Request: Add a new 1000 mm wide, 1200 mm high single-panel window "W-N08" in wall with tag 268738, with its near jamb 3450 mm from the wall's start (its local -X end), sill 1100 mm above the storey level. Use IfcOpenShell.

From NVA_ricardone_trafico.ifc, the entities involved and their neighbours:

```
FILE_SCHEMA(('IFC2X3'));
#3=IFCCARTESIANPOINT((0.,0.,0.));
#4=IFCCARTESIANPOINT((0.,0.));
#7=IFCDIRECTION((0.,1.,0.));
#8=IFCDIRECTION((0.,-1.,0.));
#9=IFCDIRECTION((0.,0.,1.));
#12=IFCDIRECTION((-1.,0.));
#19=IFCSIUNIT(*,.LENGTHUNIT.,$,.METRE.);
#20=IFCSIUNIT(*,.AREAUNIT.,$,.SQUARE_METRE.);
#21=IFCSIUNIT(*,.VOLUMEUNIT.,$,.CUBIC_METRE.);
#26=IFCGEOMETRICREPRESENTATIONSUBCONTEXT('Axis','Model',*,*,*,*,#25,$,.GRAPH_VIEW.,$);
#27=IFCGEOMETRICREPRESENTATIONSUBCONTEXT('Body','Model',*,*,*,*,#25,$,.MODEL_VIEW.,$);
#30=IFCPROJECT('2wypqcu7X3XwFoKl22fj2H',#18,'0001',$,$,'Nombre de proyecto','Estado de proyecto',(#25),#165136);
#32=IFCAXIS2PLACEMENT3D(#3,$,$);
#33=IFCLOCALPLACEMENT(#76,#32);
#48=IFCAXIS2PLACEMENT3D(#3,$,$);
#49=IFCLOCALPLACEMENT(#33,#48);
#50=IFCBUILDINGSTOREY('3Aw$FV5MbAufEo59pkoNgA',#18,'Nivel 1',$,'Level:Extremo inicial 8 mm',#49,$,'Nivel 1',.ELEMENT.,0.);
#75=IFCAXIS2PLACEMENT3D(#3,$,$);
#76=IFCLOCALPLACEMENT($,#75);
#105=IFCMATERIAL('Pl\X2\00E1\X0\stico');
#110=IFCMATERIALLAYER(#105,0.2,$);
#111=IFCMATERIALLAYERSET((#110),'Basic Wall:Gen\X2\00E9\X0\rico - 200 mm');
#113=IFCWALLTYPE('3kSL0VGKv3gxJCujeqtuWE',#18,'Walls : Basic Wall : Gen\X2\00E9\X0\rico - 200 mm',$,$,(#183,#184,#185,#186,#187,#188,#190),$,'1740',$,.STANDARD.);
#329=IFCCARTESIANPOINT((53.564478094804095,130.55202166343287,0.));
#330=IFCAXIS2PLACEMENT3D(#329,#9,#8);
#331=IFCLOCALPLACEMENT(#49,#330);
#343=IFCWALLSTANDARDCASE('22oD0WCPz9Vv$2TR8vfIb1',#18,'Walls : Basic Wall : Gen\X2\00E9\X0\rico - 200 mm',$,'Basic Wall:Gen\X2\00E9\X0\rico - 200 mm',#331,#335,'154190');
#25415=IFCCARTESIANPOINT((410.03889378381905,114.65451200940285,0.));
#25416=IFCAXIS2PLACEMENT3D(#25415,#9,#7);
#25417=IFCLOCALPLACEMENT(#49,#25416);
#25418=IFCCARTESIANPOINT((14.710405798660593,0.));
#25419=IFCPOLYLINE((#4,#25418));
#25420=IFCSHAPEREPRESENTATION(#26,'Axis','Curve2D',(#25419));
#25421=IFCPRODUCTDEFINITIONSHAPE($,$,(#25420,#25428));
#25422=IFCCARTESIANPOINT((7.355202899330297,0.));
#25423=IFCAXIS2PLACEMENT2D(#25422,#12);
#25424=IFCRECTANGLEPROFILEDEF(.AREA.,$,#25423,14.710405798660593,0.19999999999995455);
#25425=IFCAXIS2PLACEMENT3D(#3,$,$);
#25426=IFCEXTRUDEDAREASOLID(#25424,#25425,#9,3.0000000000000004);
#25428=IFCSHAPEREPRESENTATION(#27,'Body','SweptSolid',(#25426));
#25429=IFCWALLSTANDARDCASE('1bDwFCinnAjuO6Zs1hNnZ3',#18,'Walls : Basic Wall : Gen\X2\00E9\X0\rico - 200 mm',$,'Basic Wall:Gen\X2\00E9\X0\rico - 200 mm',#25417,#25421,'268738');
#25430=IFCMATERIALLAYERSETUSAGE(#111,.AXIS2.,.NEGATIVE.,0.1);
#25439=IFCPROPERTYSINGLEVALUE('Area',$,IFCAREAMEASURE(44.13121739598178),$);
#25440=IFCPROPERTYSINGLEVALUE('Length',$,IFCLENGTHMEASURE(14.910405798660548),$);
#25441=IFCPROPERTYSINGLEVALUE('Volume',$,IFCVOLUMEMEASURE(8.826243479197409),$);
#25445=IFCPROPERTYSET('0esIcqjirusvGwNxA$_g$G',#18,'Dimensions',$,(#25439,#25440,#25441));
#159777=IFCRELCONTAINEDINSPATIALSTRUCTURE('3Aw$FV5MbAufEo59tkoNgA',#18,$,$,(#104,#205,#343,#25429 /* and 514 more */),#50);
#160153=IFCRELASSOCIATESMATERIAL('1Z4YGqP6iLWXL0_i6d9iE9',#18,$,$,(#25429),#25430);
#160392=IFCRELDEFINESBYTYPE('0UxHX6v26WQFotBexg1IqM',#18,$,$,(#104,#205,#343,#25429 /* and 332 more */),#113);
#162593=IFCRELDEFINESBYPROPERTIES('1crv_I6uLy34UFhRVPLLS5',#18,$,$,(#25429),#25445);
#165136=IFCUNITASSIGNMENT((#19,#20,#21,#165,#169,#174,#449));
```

```python
import numpy as np
import ifcopenshell
import ifcopenshell.api.feature
import ifcopenshell.api.geometry
import ifcopenshell.api.pset
import ifcopenshell.api.root
import ifcopenshell.api.spatial
import ifcopenshell.api.type
import ifcopenshell.geom
import ifcopenshell.util.element
import ifcopenshell.util.placement
import ifcopenshell.util.representation
import ifcopenshell.util.shape
import ifcopenshell.util.unit

model = ifcopenshell.open("NVA_ricardone_trafico.ifc")
unit_scale = ifcopenshell.util.unit.calculate_unit_scale(model)
area_scale = ifcopenshell.util.unit.calculate_unit_scale(model, "AREAUNIT")
volume_scale = ifcopenshell.util.unit.calculate_unit_scale(model, "VOLUMEUNIT")
settings = ifcopenshell.geom.settings()


def volume(element):
    """Net volume in cubic metres, openings subtracted."""
    shape = ifcopenshell.geom.create_shape(settings, element)
    return ifcopenshell.util.shape.get_volume(shape.geometry)


wall = model.by_guid("1bDwFCinnAjuO6Zs1hNnZ3")
storey = ifcopenshell.util.element.get_container(wall, ifc_class="IfcBuildingStorey")
context = ifcopenshell.util.representation.get_context(model, "Model", "Body", "MODEL_VIEW")
before = volume(wall)

width, height, from_end, sill = 1, 1.2, 3.45, 1.1  # metres

# The wall runs along its own X axis, and the end named is its -X end.
wall_shape = ifcopenshell.geom.create_shape(settings, wall)
x, y, z = ifcopenshell.util.shape.get_vertices(wall_shape.geometry).T
start = x.min() + from_end
face, thickness = float(y.min()), float(y.max() - y.min())
wall_matrix = ifcopenshell.util.placement.get_local_placement(wall.ObjectPlacement)
level = ifcopenshell.util.placement.get_local_placement(storey.ObjectPlacement)[2, 3]


def in_wall(x, y):
    """Placement at x, y metres in the wall's axes, at sill height."""
    matrix = wall_matrix.copy()
    matrix[:, 3] = wall_matrix @ np.array([x / unit_scale, y / unit_scale, 0.0, 1.0])
    matrix[2, 3] = level + sill / unit_scale
    return matrix


# Opening: a box that overshoots both wall faces by 50 mm.
opening = ifcopenshell.api.root.create_entity(model, ifc_class="IfcOpeningElement")
box = ifcopenshell.api.geometry.add_wall_representation(
    model, context=context, length=width, height=height, thickness=thickness + 0.1
)
ifcopenshell.api.geometry.assign_representation(model, product=opening, representation=box)
ifcopenshell.api.geometry.edit_object_placement(model, product=opening, matrix=in_wall(start, face - 0.05), is_si=False)
ifcopenshell.api.feature.add_feature(model, feature=opening, element=wall)

window = ifcopenshell.api.root.create_entity(model, ifc_class="IfcWindow", name="W-N08")
window.OverallWidth, window.OverallHeight = width / unit_scale, height / unit_scale
body = ifcopenshell.api.geometry.add_window_representation(
    model,
    context=context,
    overall_width=window.OverallWidth,
    overall_height=window.OverallHeight,
    partition_type="SINGLE_PANEL",
)
ifcopenshell.api.geometry.assign_representation(model, product=window, representation=body)
ifcopenshell.api.spatial.assign_container(model, products=[window], relating_structure=storey)
fills = ifcopenshell.api.feature.add_filling(model, opening=opening, element=window)
fills.OwnerHistory = window.OwnerHistory  # required in IFC2X3

# IFC2X3 keeps the operation on the window style.
style = ifcopenshell.api.root.create_entity(model, ifc_class="IfcWindowStyle", name="W-N08")
style.OperationType, style.ConstructionType = "SINGLE_PANEL", "NOTDEFINED"
style.ParameterTakesPrecedence = style.Sizeable = False
ifcopenshell.api.type.assign_type(model, related_objects=[window], relating_type=style)

# Centre the window in the wall's thickness.
ifcopenshell.api.geometry.edit_object_placement(model, product=window, matrix=in_wall(start, face), is_si=False)
window_shape = ifcopenshell.geom.create_shape(settings, window)
depth = ifcopenshell.util.shape.get_vertices(window_shape.geometry)[:, 1]
offset = face + thickness / 2 - (depth.min() + depth.max()) / 2
ifcopenshell.api.geometry.edit_object_placement(model, product=window, matrix=in_wall(start, offset), is_si=False)

after = volume(wall)

# Update the wall's stored quantities.
pset = model.by_id(ifcopenshell.util.element.get_pset(wall, "Dimensions", should_inherit=False)["id"])
ifcopenshell.api.pset.edit_pset(model, pset=pset, properties={
    "Area": model.create_entity("IfcAreaMeasure", after / thickness / area_scale),
    "Volume": model.create_entity("IfcVolumeMeasure", after / volume_scale),
})

print(f"wall volume {before:.3f} -> {after:.3f} m3")

model.write("NVA_ricardone_trafico_v2.ifc")
```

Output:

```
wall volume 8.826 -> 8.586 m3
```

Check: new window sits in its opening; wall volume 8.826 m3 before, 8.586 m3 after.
